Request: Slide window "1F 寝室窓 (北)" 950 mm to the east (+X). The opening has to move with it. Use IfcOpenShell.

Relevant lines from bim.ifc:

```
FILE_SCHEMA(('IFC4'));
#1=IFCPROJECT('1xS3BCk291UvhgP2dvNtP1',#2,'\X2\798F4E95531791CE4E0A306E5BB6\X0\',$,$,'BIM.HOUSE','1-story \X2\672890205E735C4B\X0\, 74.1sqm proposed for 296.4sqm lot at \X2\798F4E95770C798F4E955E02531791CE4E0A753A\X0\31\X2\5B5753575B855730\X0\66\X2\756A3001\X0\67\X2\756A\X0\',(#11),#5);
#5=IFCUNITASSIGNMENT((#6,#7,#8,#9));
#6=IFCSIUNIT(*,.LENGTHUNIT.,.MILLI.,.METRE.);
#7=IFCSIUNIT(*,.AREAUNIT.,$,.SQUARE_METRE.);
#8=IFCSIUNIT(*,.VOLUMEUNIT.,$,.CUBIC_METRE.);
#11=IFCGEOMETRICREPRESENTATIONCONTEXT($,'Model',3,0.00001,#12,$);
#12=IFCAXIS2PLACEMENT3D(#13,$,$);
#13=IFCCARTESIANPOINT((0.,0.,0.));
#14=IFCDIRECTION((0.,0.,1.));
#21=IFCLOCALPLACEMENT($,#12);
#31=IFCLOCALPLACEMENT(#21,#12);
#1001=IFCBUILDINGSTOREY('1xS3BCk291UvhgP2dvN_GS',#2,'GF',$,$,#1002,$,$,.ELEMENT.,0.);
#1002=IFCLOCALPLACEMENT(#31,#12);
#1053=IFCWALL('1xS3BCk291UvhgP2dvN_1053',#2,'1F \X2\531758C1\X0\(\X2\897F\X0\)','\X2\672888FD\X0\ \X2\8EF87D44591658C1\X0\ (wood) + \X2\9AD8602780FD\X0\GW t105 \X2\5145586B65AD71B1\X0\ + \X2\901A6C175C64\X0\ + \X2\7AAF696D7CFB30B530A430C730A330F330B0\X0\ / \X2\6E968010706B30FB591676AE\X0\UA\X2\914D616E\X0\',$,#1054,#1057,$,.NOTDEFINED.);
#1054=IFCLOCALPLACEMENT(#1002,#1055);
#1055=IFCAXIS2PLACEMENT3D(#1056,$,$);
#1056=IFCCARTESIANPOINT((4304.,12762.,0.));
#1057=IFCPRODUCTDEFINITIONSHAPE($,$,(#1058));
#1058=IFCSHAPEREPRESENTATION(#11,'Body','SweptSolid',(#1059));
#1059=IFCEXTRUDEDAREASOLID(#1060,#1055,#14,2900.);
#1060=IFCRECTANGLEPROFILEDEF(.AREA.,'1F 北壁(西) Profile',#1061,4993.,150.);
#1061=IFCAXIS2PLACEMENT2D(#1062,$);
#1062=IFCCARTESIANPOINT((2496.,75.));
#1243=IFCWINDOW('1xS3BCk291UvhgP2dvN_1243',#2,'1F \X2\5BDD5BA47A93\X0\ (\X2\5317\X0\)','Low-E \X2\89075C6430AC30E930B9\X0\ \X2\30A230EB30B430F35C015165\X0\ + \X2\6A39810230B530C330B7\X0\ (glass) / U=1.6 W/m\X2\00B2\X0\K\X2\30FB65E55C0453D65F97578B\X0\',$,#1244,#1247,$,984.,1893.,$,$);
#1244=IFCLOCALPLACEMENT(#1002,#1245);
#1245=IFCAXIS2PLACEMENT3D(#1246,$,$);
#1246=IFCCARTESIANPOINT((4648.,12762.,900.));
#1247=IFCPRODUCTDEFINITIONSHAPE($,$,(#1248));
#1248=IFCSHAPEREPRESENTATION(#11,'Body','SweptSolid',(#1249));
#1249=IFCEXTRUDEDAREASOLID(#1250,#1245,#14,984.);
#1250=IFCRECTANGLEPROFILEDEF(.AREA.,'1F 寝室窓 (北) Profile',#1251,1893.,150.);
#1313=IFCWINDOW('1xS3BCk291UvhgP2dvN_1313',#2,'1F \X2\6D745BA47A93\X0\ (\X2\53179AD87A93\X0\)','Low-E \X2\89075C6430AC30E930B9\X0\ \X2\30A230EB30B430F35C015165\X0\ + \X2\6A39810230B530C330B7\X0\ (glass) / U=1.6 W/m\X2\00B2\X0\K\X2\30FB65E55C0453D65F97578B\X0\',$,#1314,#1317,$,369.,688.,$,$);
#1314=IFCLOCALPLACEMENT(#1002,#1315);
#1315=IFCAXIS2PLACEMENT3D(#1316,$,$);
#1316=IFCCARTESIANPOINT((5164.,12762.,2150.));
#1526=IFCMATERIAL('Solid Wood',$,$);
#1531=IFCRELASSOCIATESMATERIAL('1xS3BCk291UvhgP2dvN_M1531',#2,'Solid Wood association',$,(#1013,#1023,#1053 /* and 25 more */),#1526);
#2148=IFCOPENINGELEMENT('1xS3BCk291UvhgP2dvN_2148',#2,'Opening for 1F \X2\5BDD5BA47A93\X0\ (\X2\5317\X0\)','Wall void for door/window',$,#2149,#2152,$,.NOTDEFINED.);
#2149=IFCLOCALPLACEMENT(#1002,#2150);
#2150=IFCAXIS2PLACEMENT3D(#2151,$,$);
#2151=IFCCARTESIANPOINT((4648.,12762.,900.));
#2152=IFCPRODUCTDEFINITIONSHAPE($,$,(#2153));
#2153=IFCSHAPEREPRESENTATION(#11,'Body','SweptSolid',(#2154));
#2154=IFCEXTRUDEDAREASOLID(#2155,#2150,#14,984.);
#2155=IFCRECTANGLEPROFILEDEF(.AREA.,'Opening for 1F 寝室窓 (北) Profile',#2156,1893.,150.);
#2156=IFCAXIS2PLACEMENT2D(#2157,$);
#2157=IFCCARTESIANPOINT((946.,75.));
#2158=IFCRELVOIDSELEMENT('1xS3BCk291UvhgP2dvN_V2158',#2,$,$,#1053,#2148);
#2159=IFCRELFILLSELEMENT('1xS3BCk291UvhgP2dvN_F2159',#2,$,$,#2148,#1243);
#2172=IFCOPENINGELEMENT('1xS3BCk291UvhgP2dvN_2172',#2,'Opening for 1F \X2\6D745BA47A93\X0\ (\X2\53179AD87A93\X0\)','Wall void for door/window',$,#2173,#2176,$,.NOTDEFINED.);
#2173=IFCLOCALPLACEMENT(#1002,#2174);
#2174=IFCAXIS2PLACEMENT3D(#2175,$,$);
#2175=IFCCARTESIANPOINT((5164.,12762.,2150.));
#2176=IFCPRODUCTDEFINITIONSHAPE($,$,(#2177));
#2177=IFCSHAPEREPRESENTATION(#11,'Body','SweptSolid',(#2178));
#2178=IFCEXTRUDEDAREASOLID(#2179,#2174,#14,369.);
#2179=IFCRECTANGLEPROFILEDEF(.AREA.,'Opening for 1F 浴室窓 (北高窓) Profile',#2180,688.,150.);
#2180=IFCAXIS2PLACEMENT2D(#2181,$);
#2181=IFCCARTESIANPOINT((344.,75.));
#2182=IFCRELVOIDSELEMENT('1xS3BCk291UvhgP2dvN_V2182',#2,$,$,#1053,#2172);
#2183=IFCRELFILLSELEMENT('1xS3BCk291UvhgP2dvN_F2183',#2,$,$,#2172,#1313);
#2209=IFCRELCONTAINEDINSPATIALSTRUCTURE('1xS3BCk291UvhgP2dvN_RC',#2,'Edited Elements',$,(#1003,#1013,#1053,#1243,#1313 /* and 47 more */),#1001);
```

```python
import ifcopenshell
import ifcopenshell.api.geometry
import ifcopenshell.util.placement
import ifcopenshell.util.unit

model = ifcopenshell.open("bim.ifc")
unit_scale = ifcopenshell.util.unit.calculate_unit_scale(model)

window = model.by_guid("1xS3BCk291UvhgP2dvN_1243")
opening = window.FillsVoids[0].RelatingOpeningElement
wall = opening.VoidsElements[0].RelatingBuildingElement

wall_matrix = ifcopenshell.util.placement.get_local_placement(wall.ObjectPlacement)
shift = wall_matrix[:3, 0] * 0.95 / unit_scale
before = ifcopenshell.util.placement.get_local_placement(window.ObjectPlacement)[:3, 3].copy()

# The window is not placed relative to its opening, so move both.
for product in (opening, window):
    matrix = ifcopenshell.util.placement.get_local_placement(product.ObjectPlacement)
    matrix[:3, 3] += shift
    ifcopenshell.api.geometry.edit_object_placement(model, product=product, matrix=matrix, is_si=False)

after = ifcopenshell.util.placement.get_local_placement(window.ObjectPlacement)[:3, 3]
print("window moved by", (after - before).round(3) + 0.0)

model.write("bim-out.ifc")
```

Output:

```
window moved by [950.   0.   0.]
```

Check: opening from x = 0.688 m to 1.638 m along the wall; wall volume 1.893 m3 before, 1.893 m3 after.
